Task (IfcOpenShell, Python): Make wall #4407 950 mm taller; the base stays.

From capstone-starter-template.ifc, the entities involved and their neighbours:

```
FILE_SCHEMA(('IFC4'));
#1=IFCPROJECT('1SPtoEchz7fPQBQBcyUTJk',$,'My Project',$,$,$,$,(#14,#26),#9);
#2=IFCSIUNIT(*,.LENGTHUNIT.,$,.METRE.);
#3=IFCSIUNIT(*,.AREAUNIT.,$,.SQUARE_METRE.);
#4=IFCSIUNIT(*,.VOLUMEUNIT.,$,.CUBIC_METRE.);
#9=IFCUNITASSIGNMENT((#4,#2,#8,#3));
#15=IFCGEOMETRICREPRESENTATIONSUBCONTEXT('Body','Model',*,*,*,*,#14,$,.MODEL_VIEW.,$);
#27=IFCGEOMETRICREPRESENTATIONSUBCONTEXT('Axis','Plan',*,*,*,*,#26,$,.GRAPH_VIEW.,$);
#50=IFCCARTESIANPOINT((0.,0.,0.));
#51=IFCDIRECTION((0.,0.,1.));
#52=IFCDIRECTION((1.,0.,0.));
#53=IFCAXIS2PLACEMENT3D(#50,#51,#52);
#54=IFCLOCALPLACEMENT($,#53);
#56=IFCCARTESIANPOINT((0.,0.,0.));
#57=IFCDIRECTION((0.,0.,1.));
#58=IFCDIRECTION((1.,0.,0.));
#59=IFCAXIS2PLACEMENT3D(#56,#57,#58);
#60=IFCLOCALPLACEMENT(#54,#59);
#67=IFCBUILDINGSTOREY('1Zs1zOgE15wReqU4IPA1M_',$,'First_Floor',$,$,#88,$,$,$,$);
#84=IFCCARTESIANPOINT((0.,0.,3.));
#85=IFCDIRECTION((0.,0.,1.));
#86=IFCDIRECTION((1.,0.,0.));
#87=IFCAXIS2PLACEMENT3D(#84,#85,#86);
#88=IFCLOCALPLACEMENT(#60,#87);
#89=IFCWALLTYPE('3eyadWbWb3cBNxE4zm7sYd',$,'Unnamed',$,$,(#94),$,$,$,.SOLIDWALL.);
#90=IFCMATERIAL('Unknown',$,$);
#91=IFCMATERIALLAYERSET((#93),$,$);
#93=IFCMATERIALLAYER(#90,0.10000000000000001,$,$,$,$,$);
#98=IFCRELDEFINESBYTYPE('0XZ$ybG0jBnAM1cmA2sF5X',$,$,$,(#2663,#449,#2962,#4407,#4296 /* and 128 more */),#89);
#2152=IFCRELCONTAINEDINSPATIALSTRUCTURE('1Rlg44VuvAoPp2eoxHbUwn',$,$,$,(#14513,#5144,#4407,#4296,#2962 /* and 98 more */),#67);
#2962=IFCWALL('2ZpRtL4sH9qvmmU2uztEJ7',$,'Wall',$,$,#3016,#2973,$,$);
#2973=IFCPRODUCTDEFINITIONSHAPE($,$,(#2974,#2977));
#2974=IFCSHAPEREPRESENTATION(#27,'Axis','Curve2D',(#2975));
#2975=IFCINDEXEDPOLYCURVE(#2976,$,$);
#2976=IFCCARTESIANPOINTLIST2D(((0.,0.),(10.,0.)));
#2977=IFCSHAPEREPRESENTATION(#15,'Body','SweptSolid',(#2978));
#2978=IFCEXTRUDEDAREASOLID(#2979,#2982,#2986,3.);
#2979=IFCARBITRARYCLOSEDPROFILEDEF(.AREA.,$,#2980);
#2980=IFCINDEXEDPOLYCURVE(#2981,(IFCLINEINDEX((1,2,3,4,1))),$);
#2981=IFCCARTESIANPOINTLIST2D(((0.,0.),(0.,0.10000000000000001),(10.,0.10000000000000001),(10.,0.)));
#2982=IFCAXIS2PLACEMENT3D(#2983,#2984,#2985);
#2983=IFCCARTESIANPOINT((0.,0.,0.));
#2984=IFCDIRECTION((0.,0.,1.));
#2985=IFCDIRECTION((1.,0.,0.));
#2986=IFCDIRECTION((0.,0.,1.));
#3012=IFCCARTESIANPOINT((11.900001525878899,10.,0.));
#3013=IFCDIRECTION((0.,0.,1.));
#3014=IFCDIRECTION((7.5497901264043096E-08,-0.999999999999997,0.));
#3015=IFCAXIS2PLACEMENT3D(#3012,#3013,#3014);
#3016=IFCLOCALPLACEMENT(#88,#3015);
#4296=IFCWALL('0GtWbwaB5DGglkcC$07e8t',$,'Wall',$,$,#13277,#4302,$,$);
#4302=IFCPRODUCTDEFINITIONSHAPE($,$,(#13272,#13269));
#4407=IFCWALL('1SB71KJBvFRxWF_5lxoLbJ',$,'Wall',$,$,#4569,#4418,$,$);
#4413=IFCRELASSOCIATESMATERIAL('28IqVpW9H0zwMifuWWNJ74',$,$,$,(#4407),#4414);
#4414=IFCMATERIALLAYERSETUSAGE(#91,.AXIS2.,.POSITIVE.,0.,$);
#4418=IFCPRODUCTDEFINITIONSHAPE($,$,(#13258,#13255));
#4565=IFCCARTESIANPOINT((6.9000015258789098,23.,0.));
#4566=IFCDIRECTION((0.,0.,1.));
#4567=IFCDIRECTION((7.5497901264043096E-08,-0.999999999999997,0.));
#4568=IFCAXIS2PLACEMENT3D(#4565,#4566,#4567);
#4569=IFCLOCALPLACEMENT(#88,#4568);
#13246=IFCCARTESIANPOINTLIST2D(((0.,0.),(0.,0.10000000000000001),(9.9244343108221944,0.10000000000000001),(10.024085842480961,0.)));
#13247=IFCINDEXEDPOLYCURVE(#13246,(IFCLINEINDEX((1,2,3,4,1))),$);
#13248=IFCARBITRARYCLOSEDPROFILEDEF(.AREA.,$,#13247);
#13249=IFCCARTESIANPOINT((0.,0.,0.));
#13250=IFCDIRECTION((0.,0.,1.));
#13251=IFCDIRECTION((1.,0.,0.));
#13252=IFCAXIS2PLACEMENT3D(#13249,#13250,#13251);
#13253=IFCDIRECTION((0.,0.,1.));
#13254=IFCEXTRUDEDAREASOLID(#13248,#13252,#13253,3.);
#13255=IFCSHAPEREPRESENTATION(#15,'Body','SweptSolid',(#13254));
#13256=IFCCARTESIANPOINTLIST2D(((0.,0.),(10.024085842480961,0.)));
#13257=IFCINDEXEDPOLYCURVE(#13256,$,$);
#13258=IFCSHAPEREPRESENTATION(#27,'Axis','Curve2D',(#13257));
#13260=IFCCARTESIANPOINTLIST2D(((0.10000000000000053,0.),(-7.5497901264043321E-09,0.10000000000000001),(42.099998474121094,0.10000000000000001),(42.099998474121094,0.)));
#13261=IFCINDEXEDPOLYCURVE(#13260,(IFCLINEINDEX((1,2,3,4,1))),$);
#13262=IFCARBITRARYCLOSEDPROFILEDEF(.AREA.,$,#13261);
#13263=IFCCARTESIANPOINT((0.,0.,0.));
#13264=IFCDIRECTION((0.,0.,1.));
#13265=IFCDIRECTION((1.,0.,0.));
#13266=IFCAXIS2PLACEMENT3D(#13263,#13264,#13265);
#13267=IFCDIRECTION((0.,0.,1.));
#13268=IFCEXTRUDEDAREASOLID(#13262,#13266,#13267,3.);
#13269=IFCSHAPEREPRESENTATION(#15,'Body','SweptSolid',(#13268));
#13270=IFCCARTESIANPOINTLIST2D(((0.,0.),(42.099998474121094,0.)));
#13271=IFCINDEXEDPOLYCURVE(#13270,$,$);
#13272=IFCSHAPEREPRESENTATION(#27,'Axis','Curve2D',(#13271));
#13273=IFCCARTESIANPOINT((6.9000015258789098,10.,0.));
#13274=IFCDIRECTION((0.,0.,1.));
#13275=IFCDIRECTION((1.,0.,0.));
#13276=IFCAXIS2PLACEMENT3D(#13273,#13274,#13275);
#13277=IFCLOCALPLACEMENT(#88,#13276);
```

```python
import ifcopenshell
import ifcopenshell.geom
import ifcopenshell.util.representation
import ifcopenshell.util.shape
import ifcopenshell.util.unit

model = ifcopenshell.open("capstone-starter-template.ifc")
unit_scale = ifcopenshell.util.unit.calculate_unit_scale(model)
settings = ifcopenshell.geom.settings()


def volume(element):
    """Net volume in cubic metres, openings subtracted."""
    shape = ifcopenshell.geom.create_shape(settings, element)
    return ifcopenshell.util.shape.get_volume(shape.geometry)


wall = model.by_guid("1SB71KJBvFRxWF_5lxoLbJ")
before = volume(wall)

body = ifcopenshell.util.representation.get_representation(wall, "Model", "Body")
solid = body.Items[0]
old_height = solid.Depth
solid.Depth += 0.95 / unit_scale
after = volume(wall)

print(f"height {old_height:g} -> {solid.Depth:g}, volume {before:.3f} -> {after:.3f} m3")

model.write("capstone-starter-template_rev.ifc")
```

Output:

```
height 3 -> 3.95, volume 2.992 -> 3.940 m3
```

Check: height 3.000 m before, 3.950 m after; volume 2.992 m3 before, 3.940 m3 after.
